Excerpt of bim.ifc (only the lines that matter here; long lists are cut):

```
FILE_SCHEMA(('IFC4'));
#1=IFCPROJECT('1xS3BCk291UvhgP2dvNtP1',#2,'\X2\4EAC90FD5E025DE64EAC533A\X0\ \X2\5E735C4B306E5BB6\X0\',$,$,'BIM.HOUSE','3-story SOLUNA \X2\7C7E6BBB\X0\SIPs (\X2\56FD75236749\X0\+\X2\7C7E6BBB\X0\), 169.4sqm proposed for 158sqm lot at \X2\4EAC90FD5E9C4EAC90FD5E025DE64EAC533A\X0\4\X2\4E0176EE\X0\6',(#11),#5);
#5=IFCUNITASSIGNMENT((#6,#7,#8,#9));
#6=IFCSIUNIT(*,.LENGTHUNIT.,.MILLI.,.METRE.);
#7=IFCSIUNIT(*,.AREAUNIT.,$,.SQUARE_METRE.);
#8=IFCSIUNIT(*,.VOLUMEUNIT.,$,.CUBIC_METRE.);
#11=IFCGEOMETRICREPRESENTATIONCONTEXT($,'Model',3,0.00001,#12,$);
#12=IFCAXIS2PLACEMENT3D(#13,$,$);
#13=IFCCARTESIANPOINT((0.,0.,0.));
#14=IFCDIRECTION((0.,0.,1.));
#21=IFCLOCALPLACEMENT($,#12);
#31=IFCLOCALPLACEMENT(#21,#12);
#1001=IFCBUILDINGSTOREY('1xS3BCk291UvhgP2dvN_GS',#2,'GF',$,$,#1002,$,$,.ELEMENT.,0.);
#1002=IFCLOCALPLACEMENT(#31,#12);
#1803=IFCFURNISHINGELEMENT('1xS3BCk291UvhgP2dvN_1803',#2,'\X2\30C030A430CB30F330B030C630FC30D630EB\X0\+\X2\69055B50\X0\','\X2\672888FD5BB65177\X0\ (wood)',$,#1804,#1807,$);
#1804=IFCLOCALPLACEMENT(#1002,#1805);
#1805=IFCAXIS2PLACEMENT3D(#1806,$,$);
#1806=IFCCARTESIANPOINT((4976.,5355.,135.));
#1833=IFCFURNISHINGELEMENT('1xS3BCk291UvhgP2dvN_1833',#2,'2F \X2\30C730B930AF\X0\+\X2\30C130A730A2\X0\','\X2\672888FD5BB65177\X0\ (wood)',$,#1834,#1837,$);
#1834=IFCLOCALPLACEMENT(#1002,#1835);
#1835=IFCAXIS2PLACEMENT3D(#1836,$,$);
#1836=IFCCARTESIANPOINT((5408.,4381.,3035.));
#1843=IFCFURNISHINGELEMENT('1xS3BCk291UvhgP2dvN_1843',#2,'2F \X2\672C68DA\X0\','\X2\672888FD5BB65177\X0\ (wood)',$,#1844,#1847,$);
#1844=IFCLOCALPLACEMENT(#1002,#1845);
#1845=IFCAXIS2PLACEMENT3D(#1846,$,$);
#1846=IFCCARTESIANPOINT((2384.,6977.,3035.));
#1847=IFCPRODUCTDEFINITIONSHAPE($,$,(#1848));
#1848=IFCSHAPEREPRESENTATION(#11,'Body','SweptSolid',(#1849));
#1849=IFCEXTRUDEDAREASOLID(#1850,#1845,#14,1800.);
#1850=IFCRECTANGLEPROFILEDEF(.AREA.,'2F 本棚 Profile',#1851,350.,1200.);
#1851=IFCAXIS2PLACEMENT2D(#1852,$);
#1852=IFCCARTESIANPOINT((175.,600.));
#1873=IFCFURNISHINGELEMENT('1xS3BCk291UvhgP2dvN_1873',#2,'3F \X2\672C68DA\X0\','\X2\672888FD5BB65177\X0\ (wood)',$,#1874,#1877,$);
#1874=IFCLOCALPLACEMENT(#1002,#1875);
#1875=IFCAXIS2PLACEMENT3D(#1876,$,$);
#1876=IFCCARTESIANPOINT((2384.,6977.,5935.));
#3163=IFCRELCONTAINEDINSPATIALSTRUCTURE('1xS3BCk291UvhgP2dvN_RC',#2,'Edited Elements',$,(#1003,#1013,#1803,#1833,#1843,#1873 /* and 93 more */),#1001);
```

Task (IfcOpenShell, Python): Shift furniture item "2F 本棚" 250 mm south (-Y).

```python
import ifcopenshell
import ifcopenshell.api.geometry
import ifcopenshell.util.placement

model = ifcopenshell.open("bim.ifc")

item = model.by_guid("1xS3BCk291UvhgP2dvN_1843")
matrix = ifcopenshell.util.placement.get_local_placement(item.ObjectPlacement)
matrix[1, 3] -= 250.0
ifcopenshell.api.geometry.edit_object_placement(model, product=item, matrix=matrix, is_si=False)

print(ifcopenshell.util.placement.get_local_placement(item.ObjectPlacement).round(3) + 0.0)

model.write("bim_updated.ifc")
```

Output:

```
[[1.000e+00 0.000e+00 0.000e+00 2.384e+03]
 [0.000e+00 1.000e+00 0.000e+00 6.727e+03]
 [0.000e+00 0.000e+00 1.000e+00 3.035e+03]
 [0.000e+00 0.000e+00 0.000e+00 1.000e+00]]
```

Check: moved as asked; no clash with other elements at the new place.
